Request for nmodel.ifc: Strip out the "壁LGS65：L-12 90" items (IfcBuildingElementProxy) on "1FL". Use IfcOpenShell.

First a look at what the model holds.

```python
import ifcopenshell
import ifcopenshell.util.element

model = ifcopenshell.open("nmodel.ifc")
print(model.schema)
storey = next(s for s in model.by_type("IfcBuildingStorey") if s.Name == "1FL")
proxies = [e for e in ifcopenshell.util.element.get_decomposition(storey) if e.is_a("IfcBuildingElementProxy")]
seen = {}
for e in proxies:
    element_type = ifcopenshell.util.element.get_type(e)
    name = element_type.Name if element_type not in (None, e) else None
    seen[name] = seen.get(name, 0) + 1
for name, count in sorted(seen.items(), key=str):
    print(count, "x", name)
```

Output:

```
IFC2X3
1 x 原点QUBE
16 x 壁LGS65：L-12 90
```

```python
import ifcopenshell
import ifcopenshell.api.root
import ifcopenshell.util.element

model = ifcopenshell.open("nmodel.ifc")

storey = next(s for s in model.by_type("IfcBuildingStorey") if s.Name == "1FL")
proxies = [e for e in ifcopenshell.util.element.get_decomposition(storey) if e.is_a("IfcBuildingElementProxy")]
targets = [e for e in proxies if (t := ifcopenshell.util.element.get_type(e)) not in (None, e) and t.Name == "壁LGS65：L-12 90"]

for e in targets:
    ifcopenshell.api.root.remove_product(model, product=e)
print(len(targets), "removed")

model.write("nmodel_v2.ifc")
```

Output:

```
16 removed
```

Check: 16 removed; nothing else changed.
